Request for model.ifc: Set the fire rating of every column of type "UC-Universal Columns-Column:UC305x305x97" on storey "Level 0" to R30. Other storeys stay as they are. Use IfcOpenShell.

First a look at what the model holds.

```python
import ifcopenshell
import ifcopenshell.util.element

model = ifcopenshell.open("model.ifc")
print(model.schema)
storey = next(s for s in model.by_type("IfcBuildingStorey") if s.Name == "Level 0")
columns = [e for e in ifcopenshell.util.element.get_decomposition(storey) if e.is_a("IfcColumn")]
seen = {}
for e in columns:
    element_type = ifcopenshell.util.element.get_type(e)
    key = (element_type.Name if element_type != e and element_type else None, ifcopenshell.util.element.get_pset(e, "Pset_ColumnCommon", "FireRating"))
    seen[key] = seen.get(key, 0) + 1
for (name, value), count in sorted(seen.items(), key=str):
    print(count, "x", name, "|", value)
```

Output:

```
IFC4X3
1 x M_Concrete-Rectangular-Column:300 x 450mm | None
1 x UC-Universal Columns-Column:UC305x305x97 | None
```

```python
import ifcopenshell
import ifcopenshell.api.pset
import ifcopenshell.util.element

model = ifcopenshell.open("model.ifc")

storey = next(s for s in model.by_type("IfcBuildingStorey") if s.Name == "Level 0")
columns = [e for e in ifcopenshell.util.element.get_decomposition(storey) if e.is_a("IfcColumn")]

count = 0
for e in columns:
    element_type = ifcopenshell.util.element.get_type(e)
    if element_type in (None, e) or element_type.Name != "UC-Universal Columns-Column:UC305x305x97":
        continue
    # add_pset returns the element's existing set when there is one.
    pset = ifcopenshell.api.pset.add_pset(model, product=e, name="Pset_ColumnCommon")
    ifcopenshell.api.pset.edit_pset(model, pset=pset, properties={"FireRating": "R30"})
    count += 1

print(count, "columns updated")

model.write("model_updated.ifc")
```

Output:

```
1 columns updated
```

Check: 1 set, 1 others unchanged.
